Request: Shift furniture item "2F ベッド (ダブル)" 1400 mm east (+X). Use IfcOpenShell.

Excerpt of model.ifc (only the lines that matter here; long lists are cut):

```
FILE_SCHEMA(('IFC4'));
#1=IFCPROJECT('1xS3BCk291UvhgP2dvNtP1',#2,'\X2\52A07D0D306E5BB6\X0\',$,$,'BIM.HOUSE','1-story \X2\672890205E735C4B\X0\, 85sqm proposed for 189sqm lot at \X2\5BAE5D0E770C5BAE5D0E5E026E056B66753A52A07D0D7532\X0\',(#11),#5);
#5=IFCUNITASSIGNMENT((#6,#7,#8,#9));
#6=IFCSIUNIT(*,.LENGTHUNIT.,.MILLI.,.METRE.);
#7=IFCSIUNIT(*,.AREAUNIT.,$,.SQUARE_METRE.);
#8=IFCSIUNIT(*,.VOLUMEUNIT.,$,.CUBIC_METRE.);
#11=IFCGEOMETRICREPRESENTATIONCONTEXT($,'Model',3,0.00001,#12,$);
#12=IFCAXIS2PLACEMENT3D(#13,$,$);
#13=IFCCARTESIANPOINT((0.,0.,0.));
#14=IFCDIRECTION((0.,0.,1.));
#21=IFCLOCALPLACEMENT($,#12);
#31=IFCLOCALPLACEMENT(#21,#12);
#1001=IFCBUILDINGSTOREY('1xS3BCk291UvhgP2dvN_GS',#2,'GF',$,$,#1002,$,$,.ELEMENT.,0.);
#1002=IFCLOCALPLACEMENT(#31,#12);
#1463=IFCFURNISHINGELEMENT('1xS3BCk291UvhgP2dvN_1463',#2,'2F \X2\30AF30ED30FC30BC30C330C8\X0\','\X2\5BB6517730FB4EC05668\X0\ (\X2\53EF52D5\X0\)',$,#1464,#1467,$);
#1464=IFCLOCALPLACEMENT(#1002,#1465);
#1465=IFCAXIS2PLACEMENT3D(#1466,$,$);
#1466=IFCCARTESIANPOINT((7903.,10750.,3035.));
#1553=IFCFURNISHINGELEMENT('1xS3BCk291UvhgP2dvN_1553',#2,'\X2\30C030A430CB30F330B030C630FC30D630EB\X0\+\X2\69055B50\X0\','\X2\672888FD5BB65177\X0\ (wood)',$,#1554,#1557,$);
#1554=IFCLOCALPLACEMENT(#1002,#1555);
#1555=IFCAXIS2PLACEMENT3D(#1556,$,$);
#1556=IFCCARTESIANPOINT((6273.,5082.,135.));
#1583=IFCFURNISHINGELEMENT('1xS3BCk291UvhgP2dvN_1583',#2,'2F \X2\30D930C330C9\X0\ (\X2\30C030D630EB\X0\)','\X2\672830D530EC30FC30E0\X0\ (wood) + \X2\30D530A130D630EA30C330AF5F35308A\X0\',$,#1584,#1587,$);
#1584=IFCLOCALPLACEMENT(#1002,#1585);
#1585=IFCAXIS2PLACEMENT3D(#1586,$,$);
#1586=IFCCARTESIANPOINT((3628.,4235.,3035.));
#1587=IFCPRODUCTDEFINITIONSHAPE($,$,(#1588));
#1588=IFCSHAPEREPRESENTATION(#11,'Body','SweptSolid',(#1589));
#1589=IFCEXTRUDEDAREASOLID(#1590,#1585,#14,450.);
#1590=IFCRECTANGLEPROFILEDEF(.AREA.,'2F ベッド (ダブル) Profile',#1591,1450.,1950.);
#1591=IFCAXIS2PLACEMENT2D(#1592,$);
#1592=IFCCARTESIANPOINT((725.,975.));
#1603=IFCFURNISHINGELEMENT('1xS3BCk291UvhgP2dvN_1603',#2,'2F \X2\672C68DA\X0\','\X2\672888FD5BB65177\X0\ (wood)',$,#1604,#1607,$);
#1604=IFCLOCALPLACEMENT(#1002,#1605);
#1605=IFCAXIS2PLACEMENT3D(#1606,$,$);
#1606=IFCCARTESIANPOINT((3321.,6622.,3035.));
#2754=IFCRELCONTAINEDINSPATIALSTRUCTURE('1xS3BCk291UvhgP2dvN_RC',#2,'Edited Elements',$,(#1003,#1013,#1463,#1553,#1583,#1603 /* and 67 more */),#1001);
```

```python
import ifcopenshell
import ifcopenshell.api.geometry
import ifcopenshell.util.placement
import ifcopenshell.util.unit

model = ifcopenshell.open("model.ifc")
unit_scale = ifcopenshell.util.unit.calculate_unit_scale(model)

item = model.by_guid("1xS3BCk291UvhgP2dvN_1583")
matrix = ifcopenshell.util.placement.get_local_placement(item.ObjectPlacement)
matrix[0, 3] += 1.4 / unit_scale
ifcopenshell.api.geometry.edit_object_placement(model, product=item, matrix=matrix, is_si=False)

print(ifcopenshell.util.placement.get_local_placement(item.ObjectPlacement).round(3) + 0.0)

model.write("model_rev.ifc")
```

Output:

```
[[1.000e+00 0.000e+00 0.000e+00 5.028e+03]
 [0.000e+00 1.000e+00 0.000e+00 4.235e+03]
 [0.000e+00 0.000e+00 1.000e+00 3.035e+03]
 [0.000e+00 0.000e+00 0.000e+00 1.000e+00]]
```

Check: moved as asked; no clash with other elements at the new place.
